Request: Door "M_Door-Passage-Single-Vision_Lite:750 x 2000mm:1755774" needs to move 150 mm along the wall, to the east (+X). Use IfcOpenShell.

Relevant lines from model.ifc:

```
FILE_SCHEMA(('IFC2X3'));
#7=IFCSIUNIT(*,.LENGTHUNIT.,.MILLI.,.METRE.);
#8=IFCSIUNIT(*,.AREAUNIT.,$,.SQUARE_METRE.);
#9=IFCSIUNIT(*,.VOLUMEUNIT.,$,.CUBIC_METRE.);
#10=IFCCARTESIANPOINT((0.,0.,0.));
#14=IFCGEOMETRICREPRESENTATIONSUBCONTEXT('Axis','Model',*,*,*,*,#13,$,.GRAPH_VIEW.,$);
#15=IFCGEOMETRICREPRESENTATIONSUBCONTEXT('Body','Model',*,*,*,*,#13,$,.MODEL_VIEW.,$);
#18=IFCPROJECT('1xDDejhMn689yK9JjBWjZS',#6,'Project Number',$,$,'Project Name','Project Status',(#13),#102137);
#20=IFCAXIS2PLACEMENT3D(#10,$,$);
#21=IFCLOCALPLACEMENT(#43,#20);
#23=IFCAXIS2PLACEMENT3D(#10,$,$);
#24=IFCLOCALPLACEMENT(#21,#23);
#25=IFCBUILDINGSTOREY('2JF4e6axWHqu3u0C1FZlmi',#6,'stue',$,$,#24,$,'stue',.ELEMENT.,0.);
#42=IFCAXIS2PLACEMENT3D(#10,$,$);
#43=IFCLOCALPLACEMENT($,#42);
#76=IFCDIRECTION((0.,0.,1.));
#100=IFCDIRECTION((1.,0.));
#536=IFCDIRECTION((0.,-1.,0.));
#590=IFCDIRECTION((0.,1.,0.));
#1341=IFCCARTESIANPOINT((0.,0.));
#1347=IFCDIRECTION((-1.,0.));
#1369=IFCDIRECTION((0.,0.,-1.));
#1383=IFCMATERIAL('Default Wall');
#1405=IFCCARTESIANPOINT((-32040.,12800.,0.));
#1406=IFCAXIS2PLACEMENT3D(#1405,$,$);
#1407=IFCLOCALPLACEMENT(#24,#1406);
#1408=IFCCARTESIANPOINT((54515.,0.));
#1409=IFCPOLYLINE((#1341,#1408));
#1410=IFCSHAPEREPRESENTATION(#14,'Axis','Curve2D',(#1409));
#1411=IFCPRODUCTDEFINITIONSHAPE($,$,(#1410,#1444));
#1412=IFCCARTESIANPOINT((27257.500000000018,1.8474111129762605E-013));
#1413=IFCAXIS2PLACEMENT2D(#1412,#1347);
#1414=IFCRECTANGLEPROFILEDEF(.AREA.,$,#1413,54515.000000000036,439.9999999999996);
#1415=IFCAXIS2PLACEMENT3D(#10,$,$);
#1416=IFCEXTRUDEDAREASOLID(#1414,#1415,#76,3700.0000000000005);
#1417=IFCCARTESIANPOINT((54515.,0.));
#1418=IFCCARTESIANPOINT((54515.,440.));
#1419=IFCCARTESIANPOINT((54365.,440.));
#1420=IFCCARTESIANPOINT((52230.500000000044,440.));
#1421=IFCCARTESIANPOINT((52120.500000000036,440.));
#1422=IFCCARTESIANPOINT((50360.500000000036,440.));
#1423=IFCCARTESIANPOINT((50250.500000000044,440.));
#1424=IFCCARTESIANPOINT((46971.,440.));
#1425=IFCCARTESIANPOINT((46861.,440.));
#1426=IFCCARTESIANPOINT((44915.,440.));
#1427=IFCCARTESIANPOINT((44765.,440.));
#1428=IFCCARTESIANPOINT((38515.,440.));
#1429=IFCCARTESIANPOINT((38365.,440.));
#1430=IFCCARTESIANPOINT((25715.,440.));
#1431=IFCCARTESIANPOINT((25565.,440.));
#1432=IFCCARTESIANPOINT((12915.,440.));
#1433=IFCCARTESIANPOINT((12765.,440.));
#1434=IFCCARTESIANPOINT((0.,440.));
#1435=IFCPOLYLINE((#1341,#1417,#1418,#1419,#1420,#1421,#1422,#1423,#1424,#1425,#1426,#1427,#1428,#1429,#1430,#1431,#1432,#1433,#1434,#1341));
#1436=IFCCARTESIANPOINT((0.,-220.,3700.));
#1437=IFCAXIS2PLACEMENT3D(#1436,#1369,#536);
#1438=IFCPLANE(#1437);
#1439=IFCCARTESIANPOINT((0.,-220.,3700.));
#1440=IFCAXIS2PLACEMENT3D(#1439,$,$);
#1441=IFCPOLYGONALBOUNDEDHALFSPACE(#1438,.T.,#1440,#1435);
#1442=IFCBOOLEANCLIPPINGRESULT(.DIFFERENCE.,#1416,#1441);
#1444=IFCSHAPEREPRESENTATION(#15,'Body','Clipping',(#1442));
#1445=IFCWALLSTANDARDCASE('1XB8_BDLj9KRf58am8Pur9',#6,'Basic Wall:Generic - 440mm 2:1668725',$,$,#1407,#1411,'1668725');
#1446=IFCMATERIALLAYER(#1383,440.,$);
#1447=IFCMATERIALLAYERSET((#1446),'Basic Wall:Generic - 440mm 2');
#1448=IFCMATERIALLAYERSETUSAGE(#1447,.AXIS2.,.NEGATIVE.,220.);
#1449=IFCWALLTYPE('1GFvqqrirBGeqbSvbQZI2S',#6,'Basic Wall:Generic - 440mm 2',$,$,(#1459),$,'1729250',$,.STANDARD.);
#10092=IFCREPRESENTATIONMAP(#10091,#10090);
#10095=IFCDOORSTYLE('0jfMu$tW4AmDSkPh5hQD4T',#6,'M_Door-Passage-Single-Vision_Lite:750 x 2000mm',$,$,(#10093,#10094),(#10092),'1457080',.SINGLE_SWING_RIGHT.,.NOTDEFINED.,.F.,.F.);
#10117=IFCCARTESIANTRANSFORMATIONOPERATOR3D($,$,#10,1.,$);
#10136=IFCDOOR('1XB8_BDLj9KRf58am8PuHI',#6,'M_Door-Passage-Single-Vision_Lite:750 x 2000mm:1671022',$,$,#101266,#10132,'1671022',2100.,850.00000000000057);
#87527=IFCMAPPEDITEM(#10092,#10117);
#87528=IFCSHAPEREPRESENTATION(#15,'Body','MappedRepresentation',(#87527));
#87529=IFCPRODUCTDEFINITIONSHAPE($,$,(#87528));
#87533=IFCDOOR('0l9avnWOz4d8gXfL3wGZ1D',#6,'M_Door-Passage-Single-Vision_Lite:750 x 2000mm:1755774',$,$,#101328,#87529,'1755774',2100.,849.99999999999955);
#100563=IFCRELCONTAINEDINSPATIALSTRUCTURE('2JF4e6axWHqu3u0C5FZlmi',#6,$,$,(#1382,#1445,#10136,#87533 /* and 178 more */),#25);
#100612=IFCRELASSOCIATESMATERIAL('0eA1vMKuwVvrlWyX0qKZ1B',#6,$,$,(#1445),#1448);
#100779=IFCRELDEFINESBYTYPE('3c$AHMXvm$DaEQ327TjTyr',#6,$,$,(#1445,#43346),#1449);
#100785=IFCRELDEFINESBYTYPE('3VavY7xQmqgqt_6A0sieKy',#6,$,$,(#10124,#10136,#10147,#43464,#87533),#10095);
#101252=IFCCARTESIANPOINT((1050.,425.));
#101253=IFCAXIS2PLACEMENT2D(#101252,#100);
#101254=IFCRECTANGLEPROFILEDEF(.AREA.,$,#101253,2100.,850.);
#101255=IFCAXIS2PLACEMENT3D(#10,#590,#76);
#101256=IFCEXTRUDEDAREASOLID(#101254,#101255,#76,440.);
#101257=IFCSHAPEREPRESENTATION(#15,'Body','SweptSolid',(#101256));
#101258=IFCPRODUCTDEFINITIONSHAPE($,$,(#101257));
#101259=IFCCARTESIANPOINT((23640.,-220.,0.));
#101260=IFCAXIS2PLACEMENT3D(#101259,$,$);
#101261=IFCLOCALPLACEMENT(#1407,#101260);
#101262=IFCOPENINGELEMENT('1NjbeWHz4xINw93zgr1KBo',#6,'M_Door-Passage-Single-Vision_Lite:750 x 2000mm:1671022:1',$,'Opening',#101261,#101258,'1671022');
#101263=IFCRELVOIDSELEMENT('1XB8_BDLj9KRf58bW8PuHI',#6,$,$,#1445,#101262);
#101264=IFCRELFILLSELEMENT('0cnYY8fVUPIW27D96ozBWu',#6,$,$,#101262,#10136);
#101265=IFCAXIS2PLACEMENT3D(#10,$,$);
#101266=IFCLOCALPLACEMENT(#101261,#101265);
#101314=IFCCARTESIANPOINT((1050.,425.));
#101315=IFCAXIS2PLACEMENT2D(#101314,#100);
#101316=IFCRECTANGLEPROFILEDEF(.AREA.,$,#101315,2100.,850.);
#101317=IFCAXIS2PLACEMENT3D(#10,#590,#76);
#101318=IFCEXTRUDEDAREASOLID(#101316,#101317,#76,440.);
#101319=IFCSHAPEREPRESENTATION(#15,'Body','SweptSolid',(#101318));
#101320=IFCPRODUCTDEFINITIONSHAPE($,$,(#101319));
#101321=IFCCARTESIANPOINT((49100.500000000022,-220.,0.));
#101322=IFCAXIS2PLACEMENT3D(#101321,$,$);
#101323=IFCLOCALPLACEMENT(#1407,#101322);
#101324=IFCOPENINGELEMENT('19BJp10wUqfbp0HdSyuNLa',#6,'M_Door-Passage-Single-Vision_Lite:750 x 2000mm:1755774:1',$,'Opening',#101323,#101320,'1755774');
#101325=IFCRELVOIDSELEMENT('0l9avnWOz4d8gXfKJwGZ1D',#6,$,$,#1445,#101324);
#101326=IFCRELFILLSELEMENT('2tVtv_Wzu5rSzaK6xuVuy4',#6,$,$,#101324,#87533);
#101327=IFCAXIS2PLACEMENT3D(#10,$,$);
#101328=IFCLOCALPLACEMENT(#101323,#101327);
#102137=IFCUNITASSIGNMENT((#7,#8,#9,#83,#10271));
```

```python
import ifcopenshell
import ifcopenshell.api.geometry
import ifcopenshell.util.placement
import ifcopenshell.util.unit

model = ifcopenshell.open("model.ifc")
unit_scale = ifcopenshell.util.unit.calculate_unit_scale(model)

door = model.by_id(87533)
opening = door.FillsVoids[0].RelatingOpeningElement
wall = opening.VoidsElements[0].RelatingBuildingElement

wall_matrix = ifcopenshell.util.placement.get_local_placement(wall.ObjectPlacement)
shift = wall_matrix[:3, 0] * 0.15 / unit_scale
before = ifcopenshell.util.placement.get_local_placement(door.ObjectPlacement)[:3, 3].copy()

# The door is placed relative to its opening, so it follows when the opening moves.
matrix = ifcopenshell.util.placement.get_local_placement(opening.ObjectPlacement)
matrix[:3, 3] += shift
ifcopenshell.api.geometry.edit_object_placement(
    model, product=opening, matrix=matrix, is_si=False, should_transform_children=True
)

after = ifcopenshell.util.placement.get_local_placement(door.ObjectPlacement)[:3, 3]
print("door moved by", (after - before).round(3) + 0.0)

model.write("model_v2.ifc")
```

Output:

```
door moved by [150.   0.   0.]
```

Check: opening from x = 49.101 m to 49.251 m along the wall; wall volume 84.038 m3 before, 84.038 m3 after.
